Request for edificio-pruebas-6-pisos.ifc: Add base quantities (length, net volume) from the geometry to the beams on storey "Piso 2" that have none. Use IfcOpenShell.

First a look at what the model holds.

```python
import ifcopenshell
import ifcopenshell.util.element
import ifcopenshell.util.unit

model = ifcopenshell.open("edificio-pruebas-6-pisos.ifc")
print(model.schema)
for unit_type in ("LENGTHUNIT", "AREAUNIT", "VOLUMEUNIT"):
    print(unit_type, ifcopenshell.util.unit.calculate_unit_scale(model, unit_type))
storey = next(s for s in model.by_type("IfcBuildingStorey") if s.Name == "Piso 2")
beams = [e for e in ifcopenshell.util.element.get_decomposition(storey) if e.is_a("IfcBeam")]
for e in sorted(beams, key=lambda e: e.id()):
    print(e.id(), e.is_a(), e.Name, list(ifcopenshell.util.element.get_psets(e, qtos_only=True)), sep=" | ")
```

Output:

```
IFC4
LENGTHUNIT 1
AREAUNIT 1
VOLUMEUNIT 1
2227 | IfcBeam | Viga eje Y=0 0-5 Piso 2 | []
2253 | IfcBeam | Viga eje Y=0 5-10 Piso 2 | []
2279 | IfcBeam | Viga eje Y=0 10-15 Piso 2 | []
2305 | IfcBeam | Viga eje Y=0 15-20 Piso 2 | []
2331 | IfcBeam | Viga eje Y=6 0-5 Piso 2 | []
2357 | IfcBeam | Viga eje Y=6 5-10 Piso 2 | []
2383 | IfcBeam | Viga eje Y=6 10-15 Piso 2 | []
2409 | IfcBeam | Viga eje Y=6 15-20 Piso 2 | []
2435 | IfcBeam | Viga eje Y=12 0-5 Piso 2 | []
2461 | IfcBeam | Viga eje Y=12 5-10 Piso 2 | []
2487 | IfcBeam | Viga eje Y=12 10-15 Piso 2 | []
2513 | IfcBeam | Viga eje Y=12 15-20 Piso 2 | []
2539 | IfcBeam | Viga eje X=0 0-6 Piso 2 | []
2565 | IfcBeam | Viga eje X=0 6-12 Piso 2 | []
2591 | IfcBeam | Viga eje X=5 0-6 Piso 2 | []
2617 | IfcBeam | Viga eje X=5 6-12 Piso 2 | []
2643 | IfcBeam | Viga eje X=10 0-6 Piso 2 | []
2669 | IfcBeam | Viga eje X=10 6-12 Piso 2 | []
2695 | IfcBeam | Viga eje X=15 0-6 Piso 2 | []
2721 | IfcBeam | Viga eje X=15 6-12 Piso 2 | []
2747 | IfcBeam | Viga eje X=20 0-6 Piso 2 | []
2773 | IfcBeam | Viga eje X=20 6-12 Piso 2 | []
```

```python
import ifcopenshell
import ifcopenshell.api.pset
import ifcopenshell.geom
import ifcopenshell.util.element
import ifcopenshell.util.shape
import ifcopenshell.util.unit

model = ifcopenshell.open("edificio-pruebas-6-pisos.ifc")
unit_scale = ifcopenshell.util.unit.calculate_unit_scale(model)
volume_scale = ifcopenshell.util.unit.calculate_unit_scale(model, "VOLUMEUNIT")
settings = ifcopenshell.geom.settings()

storey = next(s for s in model.by_type("IfcBuildingStorey") if s.Name == "Piso 2")
beams = [e for e in ifcopenshell.util.element.get_decomposition(storey) if e.is_a("IfcBeam")]

for e in sorted(beams, key=lambda e: e.id()):
    if ifcopenshell.util.element.get_psets(e, qtos_only=True, should_inherit=False):
        continue
    # Geometry comes back in metres, in the element's own axes.
    shape = ifcopenshell.geom.create_shape(settings, e)
    values = {
        "Length": ifcopenshell.util.shape.get_max_xyz(shape.geometry) / unit_scale,
        "NetVolume": ifcopenshell.util.shape.get_volume(shape.geometry) / volume_scale,
    }
    qto = ifcopenshell.api.pset.add_qto(model, product=e, name="Qto_BeamBaseQuantities")
    ifcopenshell.api.pset.edit_qto(model, qto=qto, properties=values)
    print(e.id(), {k: round(v, 3) for k, v in values.items()})

model.write("edificio-pruebas-6-pisos_edited.ifc")
```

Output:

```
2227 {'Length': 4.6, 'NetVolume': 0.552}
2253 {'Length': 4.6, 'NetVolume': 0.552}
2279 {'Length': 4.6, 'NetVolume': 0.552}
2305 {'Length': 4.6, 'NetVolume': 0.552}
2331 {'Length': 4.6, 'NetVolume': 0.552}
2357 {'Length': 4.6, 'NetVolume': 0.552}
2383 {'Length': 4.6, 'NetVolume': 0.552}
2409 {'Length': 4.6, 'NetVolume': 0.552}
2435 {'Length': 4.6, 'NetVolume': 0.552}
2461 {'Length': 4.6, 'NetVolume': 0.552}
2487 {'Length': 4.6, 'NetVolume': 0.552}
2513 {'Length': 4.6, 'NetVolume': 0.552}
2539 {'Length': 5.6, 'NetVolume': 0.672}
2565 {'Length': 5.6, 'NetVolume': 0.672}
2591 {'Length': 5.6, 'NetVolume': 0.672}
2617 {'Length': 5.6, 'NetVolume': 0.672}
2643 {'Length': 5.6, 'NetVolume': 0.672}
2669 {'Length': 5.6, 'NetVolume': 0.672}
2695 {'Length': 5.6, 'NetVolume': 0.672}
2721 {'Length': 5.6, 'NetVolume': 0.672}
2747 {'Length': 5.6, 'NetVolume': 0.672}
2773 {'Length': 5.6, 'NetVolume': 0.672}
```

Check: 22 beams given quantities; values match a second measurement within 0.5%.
